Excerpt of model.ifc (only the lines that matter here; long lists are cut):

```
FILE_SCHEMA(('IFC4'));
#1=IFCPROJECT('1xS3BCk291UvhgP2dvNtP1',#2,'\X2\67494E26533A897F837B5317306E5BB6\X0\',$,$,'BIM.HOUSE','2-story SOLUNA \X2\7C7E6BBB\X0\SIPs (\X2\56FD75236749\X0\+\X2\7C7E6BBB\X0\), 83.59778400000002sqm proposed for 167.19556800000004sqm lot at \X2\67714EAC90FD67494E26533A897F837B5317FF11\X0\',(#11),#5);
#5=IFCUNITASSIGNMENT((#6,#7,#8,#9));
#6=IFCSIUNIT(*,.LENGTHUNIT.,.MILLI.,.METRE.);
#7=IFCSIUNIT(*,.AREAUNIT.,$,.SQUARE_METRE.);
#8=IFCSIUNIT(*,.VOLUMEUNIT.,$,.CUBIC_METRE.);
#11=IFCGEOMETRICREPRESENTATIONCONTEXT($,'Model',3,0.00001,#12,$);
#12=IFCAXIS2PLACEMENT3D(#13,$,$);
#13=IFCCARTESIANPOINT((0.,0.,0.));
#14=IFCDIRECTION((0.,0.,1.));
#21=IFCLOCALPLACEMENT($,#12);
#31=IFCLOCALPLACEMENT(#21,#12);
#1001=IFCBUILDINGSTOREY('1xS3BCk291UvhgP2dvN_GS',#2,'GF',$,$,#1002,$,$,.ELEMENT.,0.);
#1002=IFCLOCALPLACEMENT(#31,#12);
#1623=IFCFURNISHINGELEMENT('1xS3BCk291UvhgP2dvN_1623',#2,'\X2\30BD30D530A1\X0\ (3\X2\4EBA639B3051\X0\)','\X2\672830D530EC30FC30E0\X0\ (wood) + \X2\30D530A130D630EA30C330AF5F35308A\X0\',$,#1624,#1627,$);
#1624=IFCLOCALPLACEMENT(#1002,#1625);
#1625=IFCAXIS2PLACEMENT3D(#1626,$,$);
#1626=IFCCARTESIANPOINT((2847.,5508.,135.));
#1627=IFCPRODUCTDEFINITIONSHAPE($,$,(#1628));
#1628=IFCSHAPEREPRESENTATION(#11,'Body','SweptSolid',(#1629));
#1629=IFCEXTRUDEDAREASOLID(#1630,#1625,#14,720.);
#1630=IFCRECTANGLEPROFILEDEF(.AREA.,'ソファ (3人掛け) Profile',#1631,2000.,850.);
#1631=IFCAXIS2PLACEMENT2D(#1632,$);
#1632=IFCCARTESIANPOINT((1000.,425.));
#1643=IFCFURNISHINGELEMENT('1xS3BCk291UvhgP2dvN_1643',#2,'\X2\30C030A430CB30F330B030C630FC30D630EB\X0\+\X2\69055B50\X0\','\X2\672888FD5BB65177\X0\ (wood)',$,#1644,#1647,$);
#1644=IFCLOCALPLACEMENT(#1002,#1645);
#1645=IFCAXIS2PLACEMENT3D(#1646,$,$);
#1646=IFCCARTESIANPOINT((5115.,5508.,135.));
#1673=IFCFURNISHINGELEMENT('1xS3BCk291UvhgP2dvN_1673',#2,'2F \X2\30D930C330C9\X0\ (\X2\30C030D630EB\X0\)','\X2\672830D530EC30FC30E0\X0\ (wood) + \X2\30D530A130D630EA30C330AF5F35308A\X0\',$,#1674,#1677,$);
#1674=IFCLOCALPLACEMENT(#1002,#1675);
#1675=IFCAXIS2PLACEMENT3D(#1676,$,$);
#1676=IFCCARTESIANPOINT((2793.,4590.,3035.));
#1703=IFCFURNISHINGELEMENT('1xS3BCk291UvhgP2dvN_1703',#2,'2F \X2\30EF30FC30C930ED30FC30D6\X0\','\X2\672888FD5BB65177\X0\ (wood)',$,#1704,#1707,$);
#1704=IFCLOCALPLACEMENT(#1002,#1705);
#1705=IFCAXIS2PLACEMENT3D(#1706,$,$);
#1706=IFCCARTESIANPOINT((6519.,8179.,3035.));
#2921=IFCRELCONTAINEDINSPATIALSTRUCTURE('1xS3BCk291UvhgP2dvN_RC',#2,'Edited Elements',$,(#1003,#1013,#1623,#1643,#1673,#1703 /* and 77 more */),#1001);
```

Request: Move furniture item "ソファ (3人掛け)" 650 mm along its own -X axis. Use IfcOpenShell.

```python
import ifcopenshell
import ifcopenshell.api.geometry
import ifcopenshell.util.placement
import ifcopenshell.util.unit

model = ifcopenshell.open("model.ifc")
unit_scale = ifcopenshell.util.unit.calculate_unit_scale(model)

item = model.by_id(1623)
matrix = ifcopenshell.util.placement.get_local_placement(item.ObjectPlacement)
matrix[:3, 3] -= matrix[:3, 0] * 0.65 / unit_scale
ifcopenshell.api.geometry.edit_object_placement(model, product=item, matrix=matrix, is_si=False)

print(ifcopenshell.util.placement.get_local_placement(item.ObjectPlacement).round(3) + 0.0)

model.write("model-out.ifc")
```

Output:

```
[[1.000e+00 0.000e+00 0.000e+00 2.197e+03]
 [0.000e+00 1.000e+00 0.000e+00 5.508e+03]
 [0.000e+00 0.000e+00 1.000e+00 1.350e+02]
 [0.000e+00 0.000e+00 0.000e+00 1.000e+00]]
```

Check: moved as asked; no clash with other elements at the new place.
